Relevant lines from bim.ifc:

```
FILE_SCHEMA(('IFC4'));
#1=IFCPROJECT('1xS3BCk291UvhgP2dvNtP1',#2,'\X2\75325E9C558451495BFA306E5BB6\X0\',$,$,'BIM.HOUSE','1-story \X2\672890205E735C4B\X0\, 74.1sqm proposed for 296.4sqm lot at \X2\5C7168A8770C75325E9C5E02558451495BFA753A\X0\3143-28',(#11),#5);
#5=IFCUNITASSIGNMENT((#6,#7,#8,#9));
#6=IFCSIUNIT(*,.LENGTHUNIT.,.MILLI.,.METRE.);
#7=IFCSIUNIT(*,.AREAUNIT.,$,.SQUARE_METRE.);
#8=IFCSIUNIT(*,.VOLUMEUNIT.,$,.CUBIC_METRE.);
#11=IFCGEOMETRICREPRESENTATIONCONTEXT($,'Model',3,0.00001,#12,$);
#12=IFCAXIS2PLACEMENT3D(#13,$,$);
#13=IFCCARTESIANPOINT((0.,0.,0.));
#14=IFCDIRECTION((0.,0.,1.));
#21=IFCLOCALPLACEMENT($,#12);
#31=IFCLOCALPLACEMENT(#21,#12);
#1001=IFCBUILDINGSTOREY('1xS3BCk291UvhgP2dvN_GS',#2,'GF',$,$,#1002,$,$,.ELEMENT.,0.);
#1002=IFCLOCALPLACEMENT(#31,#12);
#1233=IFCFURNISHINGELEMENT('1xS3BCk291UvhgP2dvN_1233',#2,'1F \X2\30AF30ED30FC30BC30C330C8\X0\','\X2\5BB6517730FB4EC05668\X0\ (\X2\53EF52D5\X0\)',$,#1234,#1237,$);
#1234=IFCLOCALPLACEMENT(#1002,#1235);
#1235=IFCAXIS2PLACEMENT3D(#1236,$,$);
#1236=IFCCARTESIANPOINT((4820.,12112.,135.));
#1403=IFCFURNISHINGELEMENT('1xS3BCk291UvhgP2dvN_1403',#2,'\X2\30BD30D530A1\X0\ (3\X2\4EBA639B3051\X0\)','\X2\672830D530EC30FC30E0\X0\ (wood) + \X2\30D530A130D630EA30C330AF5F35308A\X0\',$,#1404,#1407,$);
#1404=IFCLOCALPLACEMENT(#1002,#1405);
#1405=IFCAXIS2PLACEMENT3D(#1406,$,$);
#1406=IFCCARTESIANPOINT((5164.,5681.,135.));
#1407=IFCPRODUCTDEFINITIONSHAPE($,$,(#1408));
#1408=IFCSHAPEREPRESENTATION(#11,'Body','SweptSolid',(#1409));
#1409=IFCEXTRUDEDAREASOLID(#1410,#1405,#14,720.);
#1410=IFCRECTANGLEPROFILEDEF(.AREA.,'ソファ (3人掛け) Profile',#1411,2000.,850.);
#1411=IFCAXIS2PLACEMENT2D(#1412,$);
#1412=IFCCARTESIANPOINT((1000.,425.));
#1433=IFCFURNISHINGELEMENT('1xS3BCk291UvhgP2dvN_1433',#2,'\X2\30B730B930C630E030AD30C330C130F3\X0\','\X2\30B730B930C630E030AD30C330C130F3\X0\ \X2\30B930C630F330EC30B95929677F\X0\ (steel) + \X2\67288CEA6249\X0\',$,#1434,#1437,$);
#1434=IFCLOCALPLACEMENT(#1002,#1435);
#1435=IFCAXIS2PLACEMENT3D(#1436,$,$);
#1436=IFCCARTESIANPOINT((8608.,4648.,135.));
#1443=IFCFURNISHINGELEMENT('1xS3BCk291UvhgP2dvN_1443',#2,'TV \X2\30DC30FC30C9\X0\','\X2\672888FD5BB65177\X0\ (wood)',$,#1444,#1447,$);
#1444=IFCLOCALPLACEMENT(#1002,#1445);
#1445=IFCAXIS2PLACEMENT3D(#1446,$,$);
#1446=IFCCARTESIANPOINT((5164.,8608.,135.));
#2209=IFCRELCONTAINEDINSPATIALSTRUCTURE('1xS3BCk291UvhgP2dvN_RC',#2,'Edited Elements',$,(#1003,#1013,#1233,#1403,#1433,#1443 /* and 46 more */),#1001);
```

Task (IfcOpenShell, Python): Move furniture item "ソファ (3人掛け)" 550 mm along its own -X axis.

```python
import ifcopenshell
import ifcopenshell.api.geometry
import ifcopenshell.util.placement
import ifcopenshell.util.unit

model = ifcopenshell.open("bim.ifc")
unit_scale = ifcopenshell.util.unit.calculate_unit_scale(model)

item = model.by_guid("1xS3BCk291UvhgP2dvN_1403")
matrix = ifcopenshell.util.placement.get_local_placement(item.ObjectPlacement)
matrix[:3, 3] -= matrix[:3, 0] * 0.55 / unit_scale
ifcopenshell.api.geometry.edit_object_placement(model, product=item, matrix=matrix, is_si=False)

print(ifcopenshell.util.placement.get_local_placement(item.ObjectPlacement).round(3) + 0.0)

model.write("bim-out.ifc")
```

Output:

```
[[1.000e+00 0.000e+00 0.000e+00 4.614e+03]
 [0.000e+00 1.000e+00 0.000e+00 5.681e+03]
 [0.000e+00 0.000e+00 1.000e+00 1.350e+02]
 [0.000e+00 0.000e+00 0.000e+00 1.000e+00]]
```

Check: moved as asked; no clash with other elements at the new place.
